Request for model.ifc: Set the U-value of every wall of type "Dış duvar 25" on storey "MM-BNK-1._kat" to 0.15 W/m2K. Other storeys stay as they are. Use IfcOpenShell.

First a look at what the model holds.

```python
import ifcopenshell
import ifcopenshell.util.element

model = ifcopenshell.open("model.ifc")
print(model.schema)
storey = next(s for s in model.by_type("IfcBuildingStorey") if s.Name == "MM-BNK-1._kat")
walls = [e for e in ifcopenshell.util.element.get_decomposition(storey) if e.is_a("IfcWall")]
seen = {}
for e in walls:
    element_type = ifcopenshell.util.element.get_type(e)
    key = (element_type.Name if element_type != e and element_type else None, ifcopenshell.util.element.get_pset(e, "Pset_WallCommon", "ThermalTransmittance"))
    seen[key] = seen.get(key, 0) + 1
for (name, value), count in sorted(seen.items(), key=str):
    print(count, "x", name, "|", value)
```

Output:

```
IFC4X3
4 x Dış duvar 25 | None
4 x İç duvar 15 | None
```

```python
import ifcopenshell
import ifcopenshell.api.pset
import ifcopenshell.util.element

model = ifcopenshell.open("model.ifc")

storey = next(s for s in model.by_type("IfcBuildingStorey") if s.Name == "MM-BNK-1._kat")
walls = [e for e in ifcopenshell.util.element.get_decomposition(storey) if e.is_a("IfcWall")]

count = 0
for e in walls:
    element_type = ifcopenshell.util.element.get_type(e)
    if element_type in (None, e) or element_type.Name != "Dış duvar 25":
        continue
    # add_pset returns the element's existing set when there is one.
    pset = ifcopenshell.api.pset.add_pset(model, product=e, name="Pset_WallCommon")
    ifcopenshell.api.pset.edit_pset(model, pset=pset, properties={"ThermalTransmittance": 0.15})
    count += 1

print(count, "walls updated")

model.write("model_edited.ifc")
```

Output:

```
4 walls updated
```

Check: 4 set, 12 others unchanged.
